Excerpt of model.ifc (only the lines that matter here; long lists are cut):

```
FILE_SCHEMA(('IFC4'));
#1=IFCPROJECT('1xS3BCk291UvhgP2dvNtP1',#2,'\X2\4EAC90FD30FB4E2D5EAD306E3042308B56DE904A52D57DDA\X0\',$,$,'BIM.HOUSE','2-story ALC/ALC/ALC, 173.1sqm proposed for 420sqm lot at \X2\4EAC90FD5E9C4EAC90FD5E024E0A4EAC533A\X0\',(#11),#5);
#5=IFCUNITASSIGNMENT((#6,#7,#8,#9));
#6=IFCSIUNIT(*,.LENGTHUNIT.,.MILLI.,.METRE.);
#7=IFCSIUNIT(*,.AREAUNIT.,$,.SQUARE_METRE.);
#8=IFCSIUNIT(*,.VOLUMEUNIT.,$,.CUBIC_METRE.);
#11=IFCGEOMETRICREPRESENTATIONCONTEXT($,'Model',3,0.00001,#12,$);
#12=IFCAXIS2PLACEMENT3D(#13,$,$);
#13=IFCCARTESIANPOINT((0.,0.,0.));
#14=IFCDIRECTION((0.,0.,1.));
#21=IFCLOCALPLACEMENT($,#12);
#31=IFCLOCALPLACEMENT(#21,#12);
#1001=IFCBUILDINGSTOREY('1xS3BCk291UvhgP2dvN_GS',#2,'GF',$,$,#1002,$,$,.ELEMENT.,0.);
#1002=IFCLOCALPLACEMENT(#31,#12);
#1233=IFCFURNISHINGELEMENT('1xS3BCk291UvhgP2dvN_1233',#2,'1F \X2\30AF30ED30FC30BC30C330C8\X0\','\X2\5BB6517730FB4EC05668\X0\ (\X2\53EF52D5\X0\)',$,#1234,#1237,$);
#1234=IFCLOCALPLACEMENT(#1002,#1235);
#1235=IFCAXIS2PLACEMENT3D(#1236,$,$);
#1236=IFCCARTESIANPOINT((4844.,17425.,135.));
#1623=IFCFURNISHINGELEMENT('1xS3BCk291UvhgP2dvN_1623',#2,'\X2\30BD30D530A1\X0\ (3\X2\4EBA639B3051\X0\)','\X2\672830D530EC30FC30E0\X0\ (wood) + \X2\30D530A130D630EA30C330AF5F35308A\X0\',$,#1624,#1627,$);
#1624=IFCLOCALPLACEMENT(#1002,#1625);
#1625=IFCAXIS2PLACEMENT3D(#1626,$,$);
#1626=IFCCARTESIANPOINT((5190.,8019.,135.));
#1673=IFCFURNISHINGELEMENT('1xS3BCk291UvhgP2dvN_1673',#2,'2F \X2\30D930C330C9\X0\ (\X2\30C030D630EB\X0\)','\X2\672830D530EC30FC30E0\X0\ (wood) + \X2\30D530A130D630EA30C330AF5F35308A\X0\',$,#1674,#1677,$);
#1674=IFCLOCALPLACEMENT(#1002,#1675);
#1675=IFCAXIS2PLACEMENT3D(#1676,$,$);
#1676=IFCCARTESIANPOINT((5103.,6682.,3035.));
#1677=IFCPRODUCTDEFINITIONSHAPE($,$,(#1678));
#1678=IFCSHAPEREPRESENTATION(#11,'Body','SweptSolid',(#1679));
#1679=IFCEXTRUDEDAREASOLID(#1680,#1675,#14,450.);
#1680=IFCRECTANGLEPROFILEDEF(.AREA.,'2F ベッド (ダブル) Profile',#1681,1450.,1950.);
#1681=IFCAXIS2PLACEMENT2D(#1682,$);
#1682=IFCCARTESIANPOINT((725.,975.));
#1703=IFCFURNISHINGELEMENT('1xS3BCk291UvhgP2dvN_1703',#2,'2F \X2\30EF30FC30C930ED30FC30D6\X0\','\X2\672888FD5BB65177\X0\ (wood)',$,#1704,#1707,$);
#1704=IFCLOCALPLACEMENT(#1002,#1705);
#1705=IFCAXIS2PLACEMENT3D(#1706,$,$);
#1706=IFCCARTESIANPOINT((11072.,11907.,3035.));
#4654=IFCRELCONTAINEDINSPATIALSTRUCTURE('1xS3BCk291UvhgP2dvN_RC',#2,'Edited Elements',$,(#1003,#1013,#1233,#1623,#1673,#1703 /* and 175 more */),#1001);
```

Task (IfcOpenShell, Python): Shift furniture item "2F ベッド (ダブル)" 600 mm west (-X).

```python
import ifcopenshell
import ifcopenshell.api.geometry
import ifcopenshell.util.placement

model = ifcopenshell.open("model.ifc")

item = model.by_guid("1xS3BCk291UvhgP2dvN_1673")
matrix = ifcopenshell.util.placement.get_local_placement(item.ObjectPlacement)
matrix[0, 3] -= 600.0
ifcopenshell.api.geometry.edit_object_placement(model, product=item, matrix=matrix, is_si=False)

print(ifcopenshell.util.placement.get_local_placement(item.ObjectPlacement).round(3) + 0.0)

model.write("model_v2.ifc")
```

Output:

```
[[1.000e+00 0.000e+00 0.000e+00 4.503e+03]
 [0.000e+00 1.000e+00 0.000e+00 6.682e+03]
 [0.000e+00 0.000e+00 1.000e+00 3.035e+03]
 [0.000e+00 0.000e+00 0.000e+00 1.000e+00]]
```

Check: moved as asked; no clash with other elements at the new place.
